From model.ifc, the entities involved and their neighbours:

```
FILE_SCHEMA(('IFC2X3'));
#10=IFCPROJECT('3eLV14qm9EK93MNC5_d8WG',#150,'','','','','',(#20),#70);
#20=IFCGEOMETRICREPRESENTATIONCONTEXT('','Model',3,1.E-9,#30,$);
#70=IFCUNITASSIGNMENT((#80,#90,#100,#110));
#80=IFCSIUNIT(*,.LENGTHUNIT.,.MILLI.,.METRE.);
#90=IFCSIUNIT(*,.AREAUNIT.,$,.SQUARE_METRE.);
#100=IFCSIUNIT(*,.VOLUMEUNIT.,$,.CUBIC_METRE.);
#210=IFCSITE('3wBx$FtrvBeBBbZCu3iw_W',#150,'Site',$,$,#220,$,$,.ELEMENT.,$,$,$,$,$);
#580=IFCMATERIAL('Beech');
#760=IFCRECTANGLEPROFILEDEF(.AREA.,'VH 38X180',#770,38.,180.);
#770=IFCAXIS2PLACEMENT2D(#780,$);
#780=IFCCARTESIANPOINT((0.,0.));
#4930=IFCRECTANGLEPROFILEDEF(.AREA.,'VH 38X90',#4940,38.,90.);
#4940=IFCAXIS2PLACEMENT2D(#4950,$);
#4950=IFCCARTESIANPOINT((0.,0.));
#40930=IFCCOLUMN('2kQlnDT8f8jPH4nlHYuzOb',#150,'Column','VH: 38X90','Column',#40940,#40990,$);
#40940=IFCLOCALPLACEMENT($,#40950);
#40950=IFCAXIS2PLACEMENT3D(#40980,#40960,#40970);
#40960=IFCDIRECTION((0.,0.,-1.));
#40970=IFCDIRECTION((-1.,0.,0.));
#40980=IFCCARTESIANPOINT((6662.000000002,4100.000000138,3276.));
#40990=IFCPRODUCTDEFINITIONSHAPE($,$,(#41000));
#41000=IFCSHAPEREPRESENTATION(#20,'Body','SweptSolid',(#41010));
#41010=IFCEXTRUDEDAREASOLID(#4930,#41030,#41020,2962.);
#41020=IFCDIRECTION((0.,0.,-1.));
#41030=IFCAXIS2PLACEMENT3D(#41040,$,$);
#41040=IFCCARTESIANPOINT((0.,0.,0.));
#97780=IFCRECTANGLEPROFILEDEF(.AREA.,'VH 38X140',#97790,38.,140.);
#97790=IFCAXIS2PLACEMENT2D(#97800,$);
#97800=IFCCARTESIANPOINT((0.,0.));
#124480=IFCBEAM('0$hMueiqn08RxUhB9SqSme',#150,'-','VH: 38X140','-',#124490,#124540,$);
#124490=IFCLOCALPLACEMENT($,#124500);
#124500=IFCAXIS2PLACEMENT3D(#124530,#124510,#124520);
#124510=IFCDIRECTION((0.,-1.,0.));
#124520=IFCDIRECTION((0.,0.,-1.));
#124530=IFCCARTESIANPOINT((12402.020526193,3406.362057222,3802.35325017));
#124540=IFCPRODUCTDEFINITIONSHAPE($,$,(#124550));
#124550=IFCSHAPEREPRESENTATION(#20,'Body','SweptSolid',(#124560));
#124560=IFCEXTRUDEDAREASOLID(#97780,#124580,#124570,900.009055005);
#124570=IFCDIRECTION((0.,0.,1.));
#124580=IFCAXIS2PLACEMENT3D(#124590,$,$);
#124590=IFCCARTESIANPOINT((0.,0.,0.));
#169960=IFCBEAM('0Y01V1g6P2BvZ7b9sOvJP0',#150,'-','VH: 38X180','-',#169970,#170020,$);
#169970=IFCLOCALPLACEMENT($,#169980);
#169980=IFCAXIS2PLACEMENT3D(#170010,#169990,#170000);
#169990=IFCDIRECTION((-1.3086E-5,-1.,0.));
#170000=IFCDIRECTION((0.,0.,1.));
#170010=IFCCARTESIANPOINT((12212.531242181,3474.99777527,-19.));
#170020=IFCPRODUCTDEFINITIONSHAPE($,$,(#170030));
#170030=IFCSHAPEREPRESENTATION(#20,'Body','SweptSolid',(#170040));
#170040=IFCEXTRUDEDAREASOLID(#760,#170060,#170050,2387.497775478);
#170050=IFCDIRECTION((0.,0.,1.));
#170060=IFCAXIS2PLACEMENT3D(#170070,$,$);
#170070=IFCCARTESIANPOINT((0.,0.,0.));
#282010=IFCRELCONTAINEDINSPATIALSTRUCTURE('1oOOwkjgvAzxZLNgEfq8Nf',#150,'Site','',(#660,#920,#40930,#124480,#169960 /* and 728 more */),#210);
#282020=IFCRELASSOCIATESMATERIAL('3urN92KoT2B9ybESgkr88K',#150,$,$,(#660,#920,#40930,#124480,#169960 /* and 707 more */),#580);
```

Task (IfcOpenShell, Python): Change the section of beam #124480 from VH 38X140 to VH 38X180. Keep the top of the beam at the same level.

```python
import ifcopenshell
import ifcopenshell.util.element

model = ifcopenshell.open("model.ifc")

member = model.by_guid("0$hMueiqn08RxUhB9SqSme")
source = next(p for p in model.by_type("IfcRectangleProfileDef") if p.ProfileName == "VH 38X180")

body = next(r for r in member.Representation.Representations if r.RepresentationIdentifier == "Body")
solid = body.Items[0]
old_profile = solid.SweptArea

# Copy the section's sizes but keep this member's own profile position.
profile = ifcopenshell.util.element.copy(model, source)
# Profiles are centred, so shift by half the change in depth to hold the top.
shift = (old_profile.XDim - profile.XDim) / 2
x, y = old_profile.Position.Location.Coordinates
up = (-1.0, 0.0)  # upwards, in the solid's own plane
location = model.createIfcCartesianPoint((x + up[0] * shift, y + up[1] * shift))
profile.Position = model.createIfcAxis2Placement2D(location, old_profile.Position.RefDirection)
solid.SweptArea = profile
if not model.get_total_inverses(old_profile):
    ifcopenshell.util.element.remove_deep2(model, old_profile)

print(solid.SweptArea)

model.write("model-out.ifc")
```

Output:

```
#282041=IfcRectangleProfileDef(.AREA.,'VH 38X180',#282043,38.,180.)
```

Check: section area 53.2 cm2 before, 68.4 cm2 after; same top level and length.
